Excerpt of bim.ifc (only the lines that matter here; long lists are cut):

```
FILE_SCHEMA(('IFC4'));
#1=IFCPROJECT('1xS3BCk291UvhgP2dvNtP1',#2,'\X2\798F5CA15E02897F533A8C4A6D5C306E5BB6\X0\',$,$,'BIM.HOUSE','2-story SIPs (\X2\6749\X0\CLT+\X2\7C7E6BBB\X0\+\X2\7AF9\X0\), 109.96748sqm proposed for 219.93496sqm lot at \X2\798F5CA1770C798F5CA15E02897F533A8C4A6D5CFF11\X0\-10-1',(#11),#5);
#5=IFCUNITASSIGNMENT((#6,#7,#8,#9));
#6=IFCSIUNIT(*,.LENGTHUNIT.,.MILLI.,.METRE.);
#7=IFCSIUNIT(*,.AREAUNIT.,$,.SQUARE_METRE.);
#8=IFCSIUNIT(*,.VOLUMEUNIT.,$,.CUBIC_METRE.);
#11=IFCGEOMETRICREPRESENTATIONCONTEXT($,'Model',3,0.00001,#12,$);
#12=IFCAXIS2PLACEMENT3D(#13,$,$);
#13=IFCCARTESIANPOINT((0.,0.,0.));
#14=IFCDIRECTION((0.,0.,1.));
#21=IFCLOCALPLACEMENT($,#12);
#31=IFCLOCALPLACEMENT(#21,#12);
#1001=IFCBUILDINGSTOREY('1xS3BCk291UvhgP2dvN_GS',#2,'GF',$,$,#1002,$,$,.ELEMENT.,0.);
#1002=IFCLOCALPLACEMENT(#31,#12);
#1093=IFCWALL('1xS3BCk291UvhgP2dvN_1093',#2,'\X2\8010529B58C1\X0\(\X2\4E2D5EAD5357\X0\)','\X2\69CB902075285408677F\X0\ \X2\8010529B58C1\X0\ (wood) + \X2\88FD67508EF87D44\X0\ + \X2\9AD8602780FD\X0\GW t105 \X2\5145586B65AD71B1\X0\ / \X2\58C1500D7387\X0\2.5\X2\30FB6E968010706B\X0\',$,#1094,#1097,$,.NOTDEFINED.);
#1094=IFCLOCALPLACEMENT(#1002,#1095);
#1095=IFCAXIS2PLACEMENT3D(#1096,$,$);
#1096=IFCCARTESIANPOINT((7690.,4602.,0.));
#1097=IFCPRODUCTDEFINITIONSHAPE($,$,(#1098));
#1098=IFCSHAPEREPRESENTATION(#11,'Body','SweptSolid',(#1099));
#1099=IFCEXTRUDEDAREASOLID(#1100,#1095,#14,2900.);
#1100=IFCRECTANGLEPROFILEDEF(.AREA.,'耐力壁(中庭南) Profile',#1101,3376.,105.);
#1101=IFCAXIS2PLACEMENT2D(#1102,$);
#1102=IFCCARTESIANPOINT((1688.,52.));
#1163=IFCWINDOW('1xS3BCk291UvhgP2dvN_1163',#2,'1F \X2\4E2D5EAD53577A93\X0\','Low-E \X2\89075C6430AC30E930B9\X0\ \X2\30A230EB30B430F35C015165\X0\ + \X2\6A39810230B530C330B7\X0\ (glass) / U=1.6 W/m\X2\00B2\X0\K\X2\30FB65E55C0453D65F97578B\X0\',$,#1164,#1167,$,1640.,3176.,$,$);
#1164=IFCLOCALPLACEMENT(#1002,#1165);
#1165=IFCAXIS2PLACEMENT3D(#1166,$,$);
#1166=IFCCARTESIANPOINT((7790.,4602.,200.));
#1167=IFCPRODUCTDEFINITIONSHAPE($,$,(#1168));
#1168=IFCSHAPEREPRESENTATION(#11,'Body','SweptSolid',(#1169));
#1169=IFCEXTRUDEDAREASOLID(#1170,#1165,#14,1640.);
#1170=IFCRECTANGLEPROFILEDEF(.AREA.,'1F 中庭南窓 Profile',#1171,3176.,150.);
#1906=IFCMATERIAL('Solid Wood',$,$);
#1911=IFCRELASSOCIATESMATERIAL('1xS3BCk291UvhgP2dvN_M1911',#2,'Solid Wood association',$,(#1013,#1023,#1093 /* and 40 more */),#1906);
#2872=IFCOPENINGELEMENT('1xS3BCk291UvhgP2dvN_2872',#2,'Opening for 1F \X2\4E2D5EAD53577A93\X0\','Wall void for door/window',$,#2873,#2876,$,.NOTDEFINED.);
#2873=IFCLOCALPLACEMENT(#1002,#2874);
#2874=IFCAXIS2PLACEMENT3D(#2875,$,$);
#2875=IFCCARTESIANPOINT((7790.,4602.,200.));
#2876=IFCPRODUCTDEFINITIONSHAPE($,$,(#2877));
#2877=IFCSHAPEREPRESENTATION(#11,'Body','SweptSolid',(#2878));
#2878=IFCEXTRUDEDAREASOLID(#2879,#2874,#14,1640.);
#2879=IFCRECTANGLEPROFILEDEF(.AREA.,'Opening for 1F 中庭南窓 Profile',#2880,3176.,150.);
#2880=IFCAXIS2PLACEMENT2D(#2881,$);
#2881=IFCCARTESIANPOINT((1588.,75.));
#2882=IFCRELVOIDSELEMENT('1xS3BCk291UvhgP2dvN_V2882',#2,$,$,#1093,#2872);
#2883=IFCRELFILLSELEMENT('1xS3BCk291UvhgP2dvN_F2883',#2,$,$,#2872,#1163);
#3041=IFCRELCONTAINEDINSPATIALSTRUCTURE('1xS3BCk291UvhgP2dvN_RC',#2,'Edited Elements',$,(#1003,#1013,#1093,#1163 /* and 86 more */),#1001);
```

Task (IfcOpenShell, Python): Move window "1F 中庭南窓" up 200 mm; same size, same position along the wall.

```python
import numpy as np
import ifcopenshell
import ifcopenshell.api.geometry
import ifcopenshell.util.placement
import ifcopenshell.util.unit

model = ifcopenshell.open("bim.ifc")
unit_scale = ifcopenshell.util.unit.calculate_unit_scale(model)

window = model.by_id(1163)
opening = window.FillsVoids[0].RelatingOpeningElement
dz = 200.0

shift = np.array([0.0, 0.0, dz])
# The window is not placed relative to its opening, so move both.
for product in (opening, window):
    matrix = ifcopenshell.util.placement.get_local_placement(product.ObjectPlacement)
    matrix[:3, 3] += shift
    ifcopenshell.api.geometry.edit_object_placement(model, product=product, matrix=matrix, is_si=False)

print(f"moved by {dz * unit_scale:+.3f} m")

model.write("bim_edited.ifc")
```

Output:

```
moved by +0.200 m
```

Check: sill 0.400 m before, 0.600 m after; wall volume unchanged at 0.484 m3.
